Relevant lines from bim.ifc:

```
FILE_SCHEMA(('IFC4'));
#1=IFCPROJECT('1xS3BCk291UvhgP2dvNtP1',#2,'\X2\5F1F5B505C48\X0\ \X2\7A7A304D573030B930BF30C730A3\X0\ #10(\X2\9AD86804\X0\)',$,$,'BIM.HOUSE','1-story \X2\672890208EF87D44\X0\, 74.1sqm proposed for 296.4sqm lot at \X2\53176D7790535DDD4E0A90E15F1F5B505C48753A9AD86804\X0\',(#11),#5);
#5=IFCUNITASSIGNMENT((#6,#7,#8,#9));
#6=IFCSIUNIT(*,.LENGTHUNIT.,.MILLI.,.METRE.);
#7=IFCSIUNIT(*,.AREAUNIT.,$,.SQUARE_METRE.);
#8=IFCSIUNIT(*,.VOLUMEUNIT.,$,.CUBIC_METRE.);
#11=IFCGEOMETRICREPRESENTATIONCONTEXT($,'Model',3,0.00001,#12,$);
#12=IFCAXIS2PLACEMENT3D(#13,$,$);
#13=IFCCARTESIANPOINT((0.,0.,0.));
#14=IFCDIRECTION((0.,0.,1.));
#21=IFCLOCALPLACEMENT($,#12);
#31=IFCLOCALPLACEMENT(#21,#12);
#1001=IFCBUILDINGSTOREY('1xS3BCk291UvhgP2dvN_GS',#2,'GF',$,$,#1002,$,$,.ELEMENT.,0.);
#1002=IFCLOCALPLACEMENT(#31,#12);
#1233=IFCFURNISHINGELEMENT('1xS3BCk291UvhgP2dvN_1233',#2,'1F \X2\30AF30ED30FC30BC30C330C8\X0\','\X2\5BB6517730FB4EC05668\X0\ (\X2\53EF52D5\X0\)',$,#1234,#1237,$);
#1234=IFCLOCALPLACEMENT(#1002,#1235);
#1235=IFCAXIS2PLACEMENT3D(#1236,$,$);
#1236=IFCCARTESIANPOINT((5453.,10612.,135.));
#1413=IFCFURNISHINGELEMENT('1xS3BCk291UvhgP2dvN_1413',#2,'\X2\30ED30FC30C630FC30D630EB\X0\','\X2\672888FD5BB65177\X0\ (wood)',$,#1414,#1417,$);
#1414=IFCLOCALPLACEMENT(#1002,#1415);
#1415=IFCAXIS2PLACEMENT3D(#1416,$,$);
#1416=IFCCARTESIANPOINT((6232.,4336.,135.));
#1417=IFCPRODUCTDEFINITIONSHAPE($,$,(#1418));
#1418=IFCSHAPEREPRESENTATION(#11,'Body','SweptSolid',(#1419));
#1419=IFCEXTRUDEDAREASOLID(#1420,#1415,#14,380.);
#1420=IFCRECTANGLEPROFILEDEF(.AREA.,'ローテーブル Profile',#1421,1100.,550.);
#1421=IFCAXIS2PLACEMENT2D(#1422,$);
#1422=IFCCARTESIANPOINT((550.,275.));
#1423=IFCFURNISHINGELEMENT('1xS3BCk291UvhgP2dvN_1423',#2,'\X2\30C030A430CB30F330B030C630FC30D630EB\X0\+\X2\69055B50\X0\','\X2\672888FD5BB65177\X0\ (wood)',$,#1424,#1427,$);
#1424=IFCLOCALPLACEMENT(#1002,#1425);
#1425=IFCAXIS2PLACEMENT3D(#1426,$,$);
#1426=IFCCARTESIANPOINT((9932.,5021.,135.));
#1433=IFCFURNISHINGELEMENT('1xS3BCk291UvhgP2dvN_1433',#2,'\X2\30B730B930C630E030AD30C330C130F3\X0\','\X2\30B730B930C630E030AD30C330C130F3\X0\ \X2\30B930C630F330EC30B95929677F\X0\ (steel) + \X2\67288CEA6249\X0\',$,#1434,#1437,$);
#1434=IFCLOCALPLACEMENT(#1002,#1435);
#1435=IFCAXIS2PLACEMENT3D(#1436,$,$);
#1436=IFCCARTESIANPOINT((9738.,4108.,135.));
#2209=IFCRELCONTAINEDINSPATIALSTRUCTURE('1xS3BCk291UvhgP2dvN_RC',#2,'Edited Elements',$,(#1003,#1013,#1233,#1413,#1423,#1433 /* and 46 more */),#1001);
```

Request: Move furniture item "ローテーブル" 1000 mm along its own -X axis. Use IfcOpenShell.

```python
import ifcopenshell
import ifcopenshell.api.geometry
import ifcopenshell.util.placement
import ifcopenshell.util.unit

model = ifcopenshell.open("bim.ifc")
unit_scale = ifcopenshell.util.unit.calculate_unit_scale(model)

item = model.by_guid("1xS3BCk291UvhgP2dvN_1413")
matrix = ifcopenshell.util.placement.get_local_placement(item.ObjectPlacement)
matrix[:3, 3] -= matrix[:3, 0] * 1 / unit_scale
ifcopenshell.api.geometry.edit_object_placement(model, product=item, matrix=matrix, is_si=False)

print(ifcopenshell.util.placement.get_local_placement(item.ObjectPlacement).round(3) + 0.0)

model.write("bim_v2.ifc")
```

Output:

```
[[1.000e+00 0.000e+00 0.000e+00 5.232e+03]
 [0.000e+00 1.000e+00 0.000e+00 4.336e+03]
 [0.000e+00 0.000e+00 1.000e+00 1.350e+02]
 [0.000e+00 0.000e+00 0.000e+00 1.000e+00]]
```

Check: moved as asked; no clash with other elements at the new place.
